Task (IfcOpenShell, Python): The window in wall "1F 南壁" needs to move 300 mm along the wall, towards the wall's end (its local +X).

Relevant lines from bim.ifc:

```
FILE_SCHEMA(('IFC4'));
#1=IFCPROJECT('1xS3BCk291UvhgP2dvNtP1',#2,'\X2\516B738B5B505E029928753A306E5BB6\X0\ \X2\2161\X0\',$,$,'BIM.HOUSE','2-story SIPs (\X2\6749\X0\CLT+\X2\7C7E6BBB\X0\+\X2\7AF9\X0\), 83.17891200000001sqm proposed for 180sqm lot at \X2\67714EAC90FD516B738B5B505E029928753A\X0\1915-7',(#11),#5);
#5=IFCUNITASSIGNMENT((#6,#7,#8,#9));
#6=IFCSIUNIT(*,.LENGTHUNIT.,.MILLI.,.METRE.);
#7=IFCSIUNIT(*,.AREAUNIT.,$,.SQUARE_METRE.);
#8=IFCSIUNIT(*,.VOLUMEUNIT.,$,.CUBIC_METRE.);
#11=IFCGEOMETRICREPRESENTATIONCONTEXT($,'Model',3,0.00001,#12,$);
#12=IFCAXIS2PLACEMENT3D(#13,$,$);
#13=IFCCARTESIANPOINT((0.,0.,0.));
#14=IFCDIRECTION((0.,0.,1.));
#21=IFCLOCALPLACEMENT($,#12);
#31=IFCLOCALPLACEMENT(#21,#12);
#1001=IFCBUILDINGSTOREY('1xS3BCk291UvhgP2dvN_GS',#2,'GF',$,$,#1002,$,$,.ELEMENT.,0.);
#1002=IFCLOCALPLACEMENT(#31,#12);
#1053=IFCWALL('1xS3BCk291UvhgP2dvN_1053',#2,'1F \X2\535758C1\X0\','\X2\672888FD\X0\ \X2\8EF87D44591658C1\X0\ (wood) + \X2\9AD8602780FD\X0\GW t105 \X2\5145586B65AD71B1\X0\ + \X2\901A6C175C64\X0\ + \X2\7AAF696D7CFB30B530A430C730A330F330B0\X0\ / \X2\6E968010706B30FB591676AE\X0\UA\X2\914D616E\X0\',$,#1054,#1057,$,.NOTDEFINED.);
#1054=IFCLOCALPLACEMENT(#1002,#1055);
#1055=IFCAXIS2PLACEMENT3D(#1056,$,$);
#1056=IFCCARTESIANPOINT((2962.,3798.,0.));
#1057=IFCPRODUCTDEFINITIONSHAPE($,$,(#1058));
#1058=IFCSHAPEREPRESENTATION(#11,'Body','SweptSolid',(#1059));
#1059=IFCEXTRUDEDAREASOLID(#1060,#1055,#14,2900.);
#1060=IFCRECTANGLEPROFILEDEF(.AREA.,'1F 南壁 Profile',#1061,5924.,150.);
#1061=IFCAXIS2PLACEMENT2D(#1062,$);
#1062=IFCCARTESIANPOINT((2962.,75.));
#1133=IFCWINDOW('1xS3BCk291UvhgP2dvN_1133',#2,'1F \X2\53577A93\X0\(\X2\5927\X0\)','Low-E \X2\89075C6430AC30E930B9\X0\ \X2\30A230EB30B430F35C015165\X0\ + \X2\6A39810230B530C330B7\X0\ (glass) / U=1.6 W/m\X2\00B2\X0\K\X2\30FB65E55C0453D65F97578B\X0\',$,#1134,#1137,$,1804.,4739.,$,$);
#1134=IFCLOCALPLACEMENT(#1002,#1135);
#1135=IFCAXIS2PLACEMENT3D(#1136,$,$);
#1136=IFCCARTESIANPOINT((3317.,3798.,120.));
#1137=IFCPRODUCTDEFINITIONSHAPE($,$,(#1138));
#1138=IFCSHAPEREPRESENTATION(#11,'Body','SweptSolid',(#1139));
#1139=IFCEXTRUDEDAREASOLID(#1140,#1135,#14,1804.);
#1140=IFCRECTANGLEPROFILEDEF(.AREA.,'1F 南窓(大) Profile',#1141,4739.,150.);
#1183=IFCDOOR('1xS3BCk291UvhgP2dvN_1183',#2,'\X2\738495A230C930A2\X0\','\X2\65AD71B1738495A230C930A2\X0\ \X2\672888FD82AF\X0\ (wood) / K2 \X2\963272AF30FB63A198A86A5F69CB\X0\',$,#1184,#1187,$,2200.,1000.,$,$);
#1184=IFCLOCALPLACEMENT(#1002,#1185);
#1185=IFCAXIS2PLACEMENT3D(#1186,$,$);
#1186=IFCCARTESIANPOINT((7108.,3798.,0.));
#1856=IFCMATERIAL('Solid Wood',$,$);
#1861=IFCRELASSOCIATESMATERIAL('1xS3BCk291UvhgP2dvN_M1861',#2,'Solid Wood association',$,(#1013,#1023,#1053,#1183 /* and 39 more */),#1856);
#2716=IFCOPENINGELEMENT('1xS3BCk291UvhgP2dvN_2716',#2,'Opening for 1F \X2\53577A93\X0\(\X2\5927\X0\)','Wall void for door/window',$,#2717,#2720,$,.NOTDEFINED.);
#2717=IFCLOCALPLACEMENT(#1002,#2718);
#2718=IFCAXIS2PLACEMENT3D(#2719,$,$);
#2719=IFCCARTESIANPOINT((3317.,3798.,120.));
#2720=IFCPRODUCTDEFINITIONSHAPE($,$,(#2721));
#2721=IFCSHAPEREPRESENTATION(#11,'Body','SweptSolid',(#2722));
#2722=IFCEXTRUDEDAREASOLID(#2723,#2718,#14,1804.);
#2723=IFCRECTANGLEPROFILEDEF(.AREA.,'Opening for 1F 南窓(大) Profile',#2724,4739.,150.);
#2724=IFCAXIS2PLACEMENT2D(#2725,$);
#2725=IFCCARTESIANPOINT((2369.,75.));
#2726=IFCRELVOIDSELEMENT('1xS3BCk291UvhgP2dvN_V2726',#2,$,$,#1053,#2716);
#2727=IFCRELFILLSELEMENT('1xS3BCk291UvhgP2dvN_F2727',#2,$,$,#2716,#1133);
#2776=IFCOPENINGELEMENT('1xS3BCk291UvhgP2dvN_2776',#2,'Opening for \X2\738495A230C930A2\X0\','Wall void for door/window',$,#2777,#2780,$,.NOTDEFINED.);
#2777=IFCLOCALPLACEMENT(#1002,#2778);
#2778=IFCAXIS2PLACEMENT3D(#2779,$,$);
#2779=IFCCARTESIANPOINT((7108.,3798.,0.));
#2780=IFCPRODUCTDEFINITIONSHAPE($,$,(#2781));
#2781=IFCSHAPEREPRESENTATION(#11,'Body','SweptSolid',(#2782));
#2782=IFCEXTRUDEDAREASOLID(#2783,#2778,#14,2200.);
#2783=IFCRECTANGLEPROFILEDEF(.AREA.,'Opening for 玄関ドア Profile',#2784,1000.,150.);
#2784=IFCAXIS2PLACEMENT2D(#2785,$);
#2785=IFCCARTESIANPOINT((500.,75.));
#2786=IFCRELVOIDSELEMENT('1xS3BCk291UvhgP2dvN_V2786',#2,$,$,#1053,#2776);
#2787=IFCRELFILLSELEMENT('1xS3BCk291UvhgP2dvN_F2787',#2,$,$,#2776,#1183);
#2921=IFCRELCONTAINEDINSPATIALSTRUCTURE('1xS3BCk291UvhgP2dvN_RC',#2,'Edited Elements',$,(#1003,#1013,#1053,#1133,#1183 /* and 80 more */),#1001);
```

```python
import ifcopenshell
import ifcopenshell.api.geometry
import ifcopenshell.util.placement
import ifcopenshell.util.unit

model = ifcopenshell.open("bim.ifc")
unit_scale = ifcopenshell.util.unit.calculate_unit_scale(model)

window = model.by_guid("1xS3BCk291UvhgP2dvN_1133")
opening = window.FillsVoids[0].RelatingOpeningElement
wall = opening.VoidsElements[0].RelatingBuildingElement

wall_matrix = ifcopenshell.util.placement.get_local_placement(wall.ObjectPlacement)
shift = wall_matrix[:3, 0] * 0.3 / unit_scale
before = ifcopenshell.util.placement.get_local_placement(window.ObjectPlacement)[:3, 3].copy()

# The window is not placed relative to its opening, so move both.
for product in (opening, window):
    matrix = ifcopenshell.util.placement.get_local_placement(product.ObjectPlacement)
    matrix[:3, 3] += shift
    ifcopenshell.api.geometry.edit_object_placement(model, product=product, matrix=matrix, is_si=False)

after = ifcopenshell.util.placement.get_local_placement(window.ObjectPlacement)[:3, 3]
print("window moved by", (after - before).round(3) + 0.0)

model.write("bim_rev.ifc")
```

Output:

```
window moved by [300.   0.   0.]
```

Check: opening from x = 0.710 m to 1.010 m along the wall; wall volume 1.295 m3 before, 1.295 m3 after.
